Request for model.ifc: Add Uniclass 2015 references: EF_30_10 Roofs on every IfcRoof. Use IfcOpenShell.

First a look at what the model holds.

```python
import ifcopenshell

model = ifcopenshell.open("model.ifc")
print(model.schema)
print("classifications:", [c.Name for c in model.by_type("IfcClassification")])
for ifc_class in ("IfcDoor", "IfcRoof", "IfcStair", "IfcWall", "IfcWindow"):
    print(ifc_class, len(model.by_type(ifc_class)))
```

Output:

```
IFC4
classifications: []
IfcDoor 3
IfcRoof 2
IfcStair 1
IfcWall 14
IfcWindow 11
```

```python
import ifcopenshell
import ifcopenshell.api.classification

model = ifcopenshell.open("model.ifc")

system = ifcopenshell.api.classification.add_classification(model, classification="Uniclass 2015")

codes = {
    "IfcRoof": ("EF_30_10", "Roofs"),
}
for ifc_class, (code, name) in codes.items():
    products = model.by_type(ifc_class)
    ifcopenshell.api.classification.add_reference(
        model, products=products, classification=system, identification=code, name=name
    )
    print(code, len(products))

model.write("model-out.ifc")
```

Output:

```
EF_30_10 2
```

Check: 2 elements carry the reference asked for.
